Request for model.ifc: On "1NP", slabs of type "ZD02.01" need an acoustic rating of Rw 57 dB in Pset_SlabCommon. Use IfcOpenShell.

First a look at what the model holds.

```python
import ifcopenshell
import ifcopenshell.util.element

model = ifcopenshell.open("model.ifc")
print(model.schema)
storey = next(s for s in model.by_type("IfcBuildingStorey") if s.Name == "1NP")
slabs = [e for e in ifcopenshell.util.element.get_decomposition(storey) if e.is_a("IfcSlab")]
seen = {}
for e in slabs:
    element_type = ifcopenshell.util.element.get_type(e)
    key = (element_type.Name if element_type != e and element_type else None, ifcopenshell.util.element.get_pset(e, "Pset_SlabCommon", "AcousticRating"))
    seen[key] = seen.get(key, 0) + 1
for (name, value), count in sorted(seen.items(), key=str):
    print(count, "x", name, "|", value)
```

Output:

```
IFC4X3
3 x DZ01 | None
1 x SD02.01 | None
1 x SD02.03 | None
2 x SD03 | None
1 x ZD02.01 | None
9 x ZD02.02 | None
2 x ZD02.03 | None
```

```python
import ifcopenshell
import ifcopenshell.api.pset
import ifcopenshell.util.element

model = ifcopenshell.open("model.ifc")

storey = next(s for s in model.by_type("IfcBuildingStorey") if s.Name == "1NP")
slabs = [e for e in ifcopenshell.util.element.get_decomposition(storey) if e.is_a("IfcSlab")]

count = 0
for e in slabs:
    element_type = ifcopenshell.util.element.get_type(e)
    if element_type in (None, e) or element_type.Name != "ZD02.01":
        continue
    # add_pset returns the element's existing set when there is one.
    pset = ifcopenshell.api.pset.add_pset(model, product=e, name="Pset_SlabCommon")
    ifcopenshell.api.pset.edit_pset(model, pset=pset, properties={"AcousticRating": "Rw 57 dB"})
    count += 1

print(count, "slabs updated")

model.write("model_updated.ifc")
```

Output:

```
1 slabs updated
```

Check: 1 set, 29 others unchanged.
